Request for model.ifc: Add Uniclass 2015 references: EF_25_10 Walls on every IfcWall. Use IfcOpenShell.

First a look at what the model holds.

```python
import ifcopenshell

model = ifcopenshell.open("model.ifc")
print(model.schema)
print("classifications:", [c.Name for c in model.by_type("IfcClassification")])
for ifc_class in ("IfcDoor", "IfcRoof", "IfcStair", "IfcWall", "IfcWindow"):
    print(ifc_class, len(model.by_type(ifc_class)))
```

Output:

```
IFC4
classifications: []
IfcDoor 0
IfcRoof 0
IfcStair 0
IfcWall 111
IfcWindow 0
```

```python
import ifcopenshell
import ifcopenshell.api.classification

model = ifcopenshell.open("model.ifc")

system = ifcopenshell.api.classification.add_classification(model, classification="Uniclass 2015")

codes = {
    "IfcWall": ("EF_25_10", "Walls"),
}
for ifc_class, (code, name) in codes.items():
    products = model.by_type(ifc_class)
    ifcopenshell.api.classification.add_reference(
        model, products=products, classification=system, identification=code, name=name
    )
    print(code, len(products))

model.write("model_v2.ifc")
```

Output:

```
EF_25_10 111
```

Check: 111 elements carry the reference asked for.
